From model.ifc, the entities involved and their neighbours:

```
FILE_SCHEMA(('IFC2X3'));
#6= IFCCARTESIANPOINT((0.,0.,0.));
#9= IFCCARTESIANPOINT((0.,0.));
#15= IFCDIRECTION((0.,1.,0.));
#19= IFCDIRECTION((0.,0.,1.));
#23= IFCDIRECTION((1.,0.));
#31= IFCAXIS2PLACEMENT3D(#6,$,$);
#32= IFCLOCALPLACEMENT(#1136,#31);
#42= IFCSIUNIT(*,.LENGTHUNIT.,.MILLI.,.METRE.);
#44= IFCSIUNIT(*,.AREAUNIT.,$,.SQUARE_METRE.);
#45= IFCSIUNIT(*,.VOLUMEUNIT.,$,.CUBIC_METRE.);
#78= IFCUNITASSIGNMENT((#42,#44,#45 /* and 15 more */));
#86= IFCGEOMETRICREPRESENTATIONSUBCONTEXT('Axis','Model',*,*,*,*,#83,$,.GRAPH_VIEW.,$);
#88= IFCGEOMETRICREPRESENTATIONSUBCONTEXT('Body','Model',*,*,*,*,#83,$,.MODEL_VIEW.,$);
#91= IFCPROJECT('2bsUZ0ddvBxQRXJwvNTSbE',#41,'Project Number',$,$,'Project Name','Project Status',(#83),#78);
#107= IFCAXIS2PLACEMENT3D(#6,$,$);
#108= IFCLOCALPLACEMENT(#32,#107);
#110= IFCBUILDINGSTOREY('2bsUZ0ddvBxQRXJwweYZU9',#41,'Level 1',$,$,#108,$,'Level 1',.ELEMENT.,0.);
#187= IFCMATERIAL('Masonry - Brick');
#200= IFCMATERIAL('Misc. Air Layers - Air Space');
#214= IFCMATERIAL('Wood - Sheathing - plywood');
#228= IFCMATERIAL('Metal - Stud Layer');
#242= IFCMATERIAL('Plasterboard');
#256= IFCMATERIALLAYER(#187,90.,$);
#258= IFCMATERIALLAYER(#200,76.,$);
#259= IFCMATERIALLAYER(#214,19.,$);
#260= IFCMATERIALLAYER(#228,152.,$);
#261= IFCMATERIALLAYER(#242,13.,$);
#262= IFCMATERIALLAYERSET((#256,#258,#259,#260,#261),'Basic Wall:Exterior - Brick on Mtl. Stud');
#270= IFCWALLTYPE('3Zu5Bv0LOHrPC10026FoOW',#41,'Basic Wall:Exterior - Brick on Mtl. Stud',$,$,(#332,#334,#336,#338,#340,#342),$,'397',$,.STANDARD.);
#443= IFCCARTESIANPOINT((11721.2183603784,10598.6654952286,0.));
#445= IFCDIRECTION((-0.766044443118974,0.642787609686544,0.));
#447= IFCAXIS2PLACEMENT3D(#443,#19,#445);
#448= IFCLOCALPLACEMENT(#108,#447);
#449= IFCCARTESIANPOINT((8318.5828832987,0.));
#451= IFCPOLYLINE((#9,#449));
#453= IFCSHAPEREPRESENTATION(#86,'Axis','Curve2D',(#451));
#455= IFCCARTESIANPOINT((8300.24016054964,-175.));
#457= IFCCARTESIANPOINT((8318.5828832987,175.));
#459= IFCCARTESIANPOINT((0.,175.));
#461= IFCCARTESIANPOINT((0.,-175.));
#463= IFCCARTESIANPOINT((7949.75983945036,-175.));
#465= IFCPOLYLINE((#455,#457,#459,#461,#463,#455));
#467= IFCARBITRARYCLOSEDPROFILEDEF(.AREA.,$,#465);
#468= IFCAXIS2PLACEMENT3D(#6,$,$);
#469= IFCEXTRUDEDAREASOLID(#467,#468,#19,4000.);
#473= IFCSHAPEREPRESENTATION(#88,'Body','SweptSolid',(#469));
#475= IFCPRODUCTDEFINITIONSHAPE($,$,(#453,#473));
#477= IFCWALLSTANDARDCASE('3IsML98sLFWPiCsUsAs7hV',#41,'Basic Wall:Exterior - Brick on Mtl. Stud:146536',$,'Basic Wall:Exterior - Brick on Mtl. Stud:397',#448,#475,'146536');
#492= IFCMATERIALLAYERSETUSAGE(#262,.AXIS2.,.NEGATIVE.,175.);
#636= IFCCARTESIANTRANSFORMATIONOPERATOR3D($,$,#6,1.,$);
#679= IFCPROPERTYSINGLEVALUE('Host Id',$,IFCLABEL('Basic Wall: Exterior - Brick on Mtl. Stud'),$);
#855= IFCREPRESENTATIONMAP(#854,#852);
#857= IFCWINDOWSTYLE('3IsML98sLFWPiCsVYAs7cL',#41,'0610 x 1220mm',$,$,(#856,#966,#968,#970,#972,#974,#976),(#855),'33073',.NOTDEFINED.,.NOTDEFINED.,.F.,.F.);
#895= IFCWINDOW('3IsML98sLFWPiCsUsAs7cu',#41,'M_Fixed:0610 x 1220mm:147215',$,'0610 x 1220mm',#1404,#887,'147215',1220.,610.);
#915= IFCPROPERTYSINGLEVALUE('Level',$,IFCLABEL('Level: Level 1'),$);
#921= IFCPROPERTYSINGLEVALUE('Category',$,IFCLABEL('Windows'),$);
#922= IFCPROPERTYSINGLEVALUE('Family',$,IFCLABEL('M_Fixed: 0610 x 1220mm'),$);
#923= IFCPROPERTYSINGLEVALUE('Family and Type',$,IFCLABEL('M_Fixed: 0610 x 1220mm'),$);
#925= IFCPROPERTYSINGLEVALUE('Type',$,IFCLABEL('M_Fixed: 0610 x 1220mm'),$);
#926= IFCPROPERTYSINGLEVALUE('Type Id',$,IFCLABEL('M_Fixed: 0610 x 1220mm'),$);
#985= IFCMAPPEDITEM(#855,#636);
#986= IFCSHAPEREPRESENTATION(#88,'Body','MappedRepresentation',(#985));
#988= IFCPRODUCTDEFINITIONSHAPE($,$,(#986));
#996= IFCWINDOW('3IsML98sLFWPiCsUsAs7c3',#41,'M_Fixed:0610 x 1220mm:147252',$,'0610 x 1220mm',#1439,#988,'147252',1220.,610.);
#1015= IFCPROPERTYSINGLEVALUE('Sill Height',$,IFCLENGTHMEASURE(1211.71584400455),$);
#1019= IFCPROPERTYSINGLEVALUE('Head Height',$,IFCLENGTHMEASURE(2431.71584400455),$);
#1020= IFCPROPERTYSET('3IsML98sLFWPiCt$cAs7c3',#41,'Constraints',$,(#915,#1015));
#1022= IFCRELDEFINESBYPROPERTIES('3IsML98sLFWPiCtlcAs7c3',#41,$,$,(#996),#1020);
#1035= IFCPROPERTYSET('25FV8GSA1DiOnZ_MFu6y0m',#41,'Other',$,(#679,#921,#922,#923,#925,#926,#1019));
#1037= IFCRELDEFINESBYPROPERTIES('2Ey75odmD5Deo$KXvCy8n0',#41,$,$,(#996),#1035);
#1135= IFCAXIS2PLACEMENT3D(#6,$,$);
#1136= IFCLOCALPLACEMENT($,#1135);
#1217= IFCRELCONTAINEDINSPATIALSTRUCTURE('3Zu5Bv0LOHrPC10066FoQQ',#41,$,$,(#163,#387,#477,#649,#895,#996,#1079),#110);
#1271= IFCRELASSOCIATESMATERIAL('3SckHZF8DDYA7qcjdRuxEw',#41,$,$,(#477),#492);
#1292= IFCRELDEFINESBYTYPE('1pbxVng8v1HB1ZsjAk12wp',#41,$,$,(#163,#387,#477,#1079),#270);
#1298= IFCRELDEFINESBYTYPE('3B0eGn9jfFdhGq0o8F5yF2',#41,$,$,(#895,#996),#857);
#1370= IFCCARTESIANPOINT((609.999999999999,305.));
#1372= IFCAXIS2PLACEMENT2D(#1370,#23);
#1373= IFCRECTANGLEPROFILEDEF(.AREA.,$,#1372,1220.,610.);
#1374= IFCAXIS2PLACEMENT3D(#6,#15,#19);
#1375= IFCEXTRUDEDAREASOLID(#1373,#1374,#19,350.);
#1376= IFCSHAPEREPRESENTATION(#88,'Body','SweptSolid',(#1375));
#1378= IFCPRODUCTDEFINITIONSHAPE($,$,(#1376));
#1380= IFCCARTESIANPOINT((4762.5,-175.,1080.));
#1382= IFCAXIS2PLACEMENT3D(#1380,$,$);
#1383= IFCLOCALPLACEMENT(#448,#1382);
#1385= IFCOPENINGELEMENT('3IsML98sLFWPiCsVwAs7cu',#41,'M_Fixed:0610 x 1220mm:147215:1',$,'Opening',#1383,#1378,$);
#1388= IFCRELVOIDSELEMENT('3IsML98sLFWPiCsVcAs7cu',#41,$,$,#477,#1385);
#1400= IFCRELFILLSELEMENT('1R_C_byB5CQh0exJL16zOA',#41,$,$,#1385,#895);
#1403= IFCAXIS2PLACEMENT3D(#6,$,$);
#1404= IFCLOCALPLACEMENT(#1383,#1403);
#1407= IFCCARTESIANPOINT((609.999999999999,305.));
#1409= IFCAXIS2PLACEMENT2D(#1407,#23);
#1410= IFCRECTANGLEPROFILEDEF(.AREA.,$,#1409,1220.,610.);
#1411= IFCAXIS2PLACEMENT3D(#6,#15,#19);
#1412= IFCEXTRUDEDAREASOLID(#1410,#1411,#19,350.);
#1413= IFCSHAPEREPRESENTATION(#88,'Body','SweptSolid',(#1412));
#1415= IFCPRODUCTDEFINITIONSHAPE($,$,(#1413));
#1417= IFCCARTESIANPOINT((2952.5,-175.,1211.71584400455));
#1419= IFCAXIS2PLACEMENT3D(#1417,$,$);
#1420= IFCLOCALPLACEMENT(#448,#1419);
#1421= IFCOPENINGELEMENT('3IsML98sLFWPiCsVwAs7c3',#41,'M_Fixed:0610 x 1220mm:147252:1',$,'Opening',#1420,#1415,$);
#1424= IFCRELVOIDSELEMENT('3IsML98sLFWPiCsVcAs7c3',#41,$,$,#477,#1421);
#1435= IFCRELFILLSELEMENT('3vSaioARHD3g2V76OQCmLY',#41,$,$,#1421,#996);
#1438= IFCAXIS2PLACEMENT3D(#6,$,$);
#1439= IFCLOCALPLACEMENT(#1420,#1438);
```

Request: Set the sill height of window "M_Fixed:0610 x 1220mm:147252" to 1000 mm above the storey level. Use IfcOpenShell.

```python
import numpy as np
import ifcopenshell
import ifcopenshell.api.geometry
import ifcopenshell.api.pset
import ifcopenshell.geom
import ifcopenshell.util.element
import ifcopenshell.util.placement
import ifcopenshell.util.shape
import ifcopenshell.util.unit

model = ifcopenshell.open("model.ifc")
unit_scale = ifcopenshell.util.unit.calculate_unit_scale(model)

window = model.by_id(996)
opening = window.FillsVoids[0].RelatingOpeningElement
storey = ifcopenshell.util.element.get_container(window, ifc_class="IfcBuildingStorey")
level = ifcopenshell.util.placement.get_local_placement(storey.ObjectPlacement)[2, 3]

# The opening's origin need not be at the sill, so measure its lowest point.
shape = ifcopenshell.geom.create_shape(ifcopenshell.geom.settings(), opening)
bottom = ifcopenshell.util.shape.get_shape_bottom_elevation(shape, shape.geometry) / unit_scale
dz = level + 1 / unit_scale - bottom

shift = np.array([0.0, 0.0, dz])
# The window is placed relative to its opening, so it follows when the opening moves.
matrix = ifcopenshell.util.placement.get_local_placement(opening.ObjectPlacement)
matrix[:3, 3] += shift
ifcopenshell.api.geometry.edit_object_placement(
    model, product=opening, matrix=matrix, is_si=False, should_transform_children=True
)

# Keep the stored heights in step.
pset = model.by_id(ifcopenshell.util.element.get_pset(window, "Constraints", should_inherit=False)["id"])
ifcopenshell.api.pset.edit_pset(model, pset=pset, properties={
    "Sill Height": model.create_entity("IfcLengthMeasure", ifcopenshell.util.element.get_pset(window, "Constraints", "Sill Height") + dz),
})
pset = model.by_id(ifcopenshell.util.element.get_pset(window, "Other", should_inherit=False)["id"])
ifcopenshell.api.pset.edit_pset(model, pset=pset, properties={
    "Head Height": model.create_entity("IfcLengthMeasure", ifcopenshell.util.element.get_pset(window, "Other", "Head Height") + dz),
})

print(f"moved by {dz * unit_scale:+.3f} m")

model.write("model-out.ifc")
```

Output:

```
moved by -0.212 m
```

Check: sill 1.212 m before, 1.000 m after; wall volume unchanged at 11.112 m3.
